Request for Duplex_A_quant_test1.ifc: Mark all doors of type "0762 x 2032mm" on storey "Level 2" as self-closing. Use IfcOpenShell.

First a look at what the model holds.

```python
import ifcopenshell
import ifcopenshell.util.element

model = ifcopenshell.open("Duplex_A_quant_test1.ifc")
print(model.schema)
storey = next(s for s in model.by_type("IfcBuildingStorey") if s.Name == "Level 2")
doors = [e for e in ifcopenshell.util.element.get_decomposition(storey) if e.is_a("IfcDoor")]
seen = {}
for e in doors:
    element_type = ifcopenshell.util.element.get_type(e)
    key = (element_type.Name if element_type != e and element_type else None, ifcopenshell.util.element.get_pset(e, "Pset_DoorCommon", "SelfClosing"))
    seen[key] = seen.get(key, 0) + 1
for (name, value), count in sorted(seen.items(), key=str):
    print(count, "x", name, "|", value)
```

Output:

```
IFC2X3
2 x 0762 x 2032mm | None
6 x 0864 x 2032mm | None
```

```python
import ifcopenshell
import ifcopenshell.api.pset
import ifcopenshell.util.element

model = ifcopenshell.open("Duplex_A_quant_test1.ifc")

storey = next(s for s in model.by_type("IfcBuildingStorey") if s.Name == "Level 2")
doors = [e for e in ifcopenshell.util.element.get_decomposition(storey) if e.is_a("IfcDoor")]

count = 0
for e in doors:
    element_type = ifcopenshell.util.element.get_type(e)
    if element_type in (None, e) or element_type.Name != "0762 x 2032mm":
        continue
    # add_pset returns the element's existing set when there is one.
    pset = ifcopenshell.api.pset.add_pset(model, product=e, name="Pset_DoorCommon")
    ifcopenshell.api.pset.edit_pset(model, pset=pset, properties={"SelfClosing": True})
    count += 1

print(count, "doors updated")

model.write("Duplex_A_quant_test1_edited.ifc")
```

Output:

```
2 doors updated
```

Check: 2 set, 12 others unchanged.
